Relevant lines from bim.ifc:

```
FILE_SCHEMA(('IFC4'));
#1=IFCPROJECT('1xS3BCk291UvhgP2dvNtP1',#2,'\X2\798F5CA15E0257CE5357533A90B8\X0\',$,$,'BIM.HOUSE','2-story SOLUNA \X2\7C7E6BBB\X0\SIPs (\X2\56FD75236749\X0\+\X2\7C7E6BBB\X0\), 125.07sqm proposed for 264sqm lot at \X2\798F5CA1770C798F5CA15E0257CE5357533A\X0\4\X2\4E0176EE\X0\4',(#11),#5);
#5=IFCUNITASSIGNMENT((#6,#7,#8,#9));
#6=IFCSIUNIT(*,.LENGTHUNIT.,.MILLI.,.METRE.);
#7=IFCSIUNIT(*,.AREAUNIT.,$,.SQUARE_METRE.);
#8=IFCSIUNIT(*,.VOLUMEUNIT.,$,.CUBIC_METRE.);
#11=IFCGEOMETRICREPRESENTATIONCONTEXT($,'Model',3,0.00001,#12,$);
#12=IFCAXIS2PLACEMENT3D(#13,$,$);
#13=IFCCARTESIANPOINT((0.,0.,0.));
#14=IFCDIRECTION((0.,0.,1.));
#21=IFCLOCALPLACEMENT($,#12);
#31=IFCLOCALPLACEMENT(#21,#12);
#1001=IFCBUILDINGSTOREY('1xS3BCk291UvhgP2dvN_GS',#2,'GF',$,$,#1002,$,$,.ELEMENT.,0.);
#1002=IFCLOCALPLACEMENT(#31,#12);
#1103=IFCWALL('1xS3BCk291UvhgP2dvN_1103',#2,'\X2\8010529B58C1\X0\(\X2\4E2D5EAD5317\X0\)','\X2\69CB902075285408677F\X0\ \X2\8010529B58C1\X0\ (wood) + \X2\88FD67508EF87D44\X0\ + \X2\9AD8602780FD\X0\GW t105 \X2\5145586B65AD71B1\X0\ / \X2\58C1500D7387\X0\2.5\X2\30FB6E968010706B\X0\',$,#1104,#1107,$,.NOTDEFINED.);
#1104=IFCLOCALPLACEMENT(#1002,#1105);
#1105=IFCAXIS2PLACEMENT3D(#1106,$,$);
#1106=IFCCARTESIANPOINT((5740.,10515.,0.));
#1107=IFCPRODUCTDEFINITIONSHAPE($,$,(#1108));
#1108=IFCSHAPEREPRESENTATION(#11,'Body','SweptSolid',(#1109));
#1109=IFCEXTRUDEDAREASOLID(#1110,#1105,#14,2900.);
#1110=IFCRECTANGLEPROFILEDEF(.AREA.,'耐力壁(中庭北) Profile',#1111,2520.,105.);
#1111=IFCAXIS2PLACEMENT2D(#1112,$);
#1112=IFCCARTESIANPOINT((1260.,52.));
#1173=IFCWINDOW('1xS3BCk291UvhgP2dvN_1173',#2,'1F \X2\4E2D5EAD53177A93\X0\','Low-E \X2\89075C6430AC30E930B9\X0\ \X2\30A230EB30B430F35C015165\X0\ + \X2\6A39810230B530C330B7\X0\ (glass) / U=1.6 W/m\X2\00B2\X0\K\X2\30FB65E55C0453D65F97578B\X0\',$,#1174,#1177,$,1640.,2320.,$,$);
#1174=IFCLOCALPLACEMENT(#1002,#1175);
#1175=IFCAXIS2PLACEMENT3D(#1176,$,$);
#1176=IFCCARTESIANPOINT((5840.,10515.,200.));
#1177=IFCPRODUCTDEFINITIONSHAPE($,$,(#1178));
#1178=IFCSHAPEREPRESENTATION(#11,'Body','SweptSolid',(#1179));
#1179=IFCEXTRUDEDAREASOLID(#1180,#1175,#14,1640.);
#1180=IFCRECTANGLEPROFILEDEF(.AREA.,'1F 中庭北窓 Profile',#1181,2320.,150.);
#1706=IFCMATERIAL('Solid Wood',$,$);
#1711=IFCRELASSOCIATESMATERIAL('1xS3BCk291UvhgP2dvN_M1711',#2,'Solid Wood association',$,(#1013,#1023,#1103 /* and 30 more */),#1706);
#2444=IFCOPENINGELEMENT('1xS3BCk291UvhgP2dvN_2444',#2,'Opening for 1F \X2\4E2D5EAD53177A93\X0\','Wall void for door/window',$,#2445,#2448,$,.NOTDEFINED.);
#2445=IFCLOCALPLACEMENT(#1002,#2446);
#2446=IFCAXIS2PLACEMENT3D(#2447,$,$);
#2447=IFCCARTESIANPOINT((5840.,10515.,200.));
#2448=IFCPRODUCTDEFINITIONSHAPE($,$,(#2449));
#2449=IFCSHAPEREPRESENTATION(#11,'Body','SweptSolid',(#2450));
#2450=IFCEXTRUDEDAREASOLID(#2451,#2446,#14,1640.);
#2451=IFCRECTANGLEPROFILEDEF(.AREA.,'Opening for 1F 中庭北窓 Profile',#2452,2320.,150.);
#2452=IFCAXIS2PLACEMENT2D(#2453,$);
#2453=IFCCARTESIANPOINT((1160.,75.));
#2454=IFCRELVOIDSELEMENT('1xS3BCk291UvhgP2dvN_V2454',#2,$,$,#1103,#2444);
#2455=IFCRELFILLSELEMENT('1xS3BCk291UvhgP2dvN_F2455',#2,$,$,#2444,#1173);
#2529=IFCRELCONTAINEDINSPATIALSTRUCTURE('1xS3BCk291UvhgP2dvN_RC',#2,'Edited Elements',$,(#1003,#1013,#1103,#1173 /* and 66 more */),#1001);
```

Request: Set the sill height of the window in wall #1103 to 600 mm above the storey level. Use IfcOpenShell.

```python
import numpy as np
import ifcopenshell
import ifcopenshell.api.geometry
import ifcopenshell.geom
import ifcopenshell.util.element
import ifcopenshell.util.placement
import ifcopenshell.util.shape
import ifcopenshell.util.unit

model = ifcopenshell.open("bim.ifc")
unit_scale = ifcopenshell.util.unit.calculate_unit_scale(model)

window = model.by_guid("1xS3BCk291UvhgP2dvN_1173")
opening = window.FillsVoids[0].RelatingOpeningElement
storey = ifcopenshell.util.element.get_container(window, ifc_class="IfcBuildingStorey")
level = ifcopenshell.util.placement.get_local_placement(storey.ObjectPlacement)[2, 3]

# The opening's origin need not be at the sill, so measure its lowest point.
shape = ifcopenshell.geom.create_shape(ifcopenshell.geom.settings(), opening)
bottom = ifcopenshell.util.shape.get_shape_bottom_elevation(shape, shape.geometry) / unit_scale
dz = level + 600.0 - bottom

shift = np.array([0.0, 0.0, dz])
# The window is not placed relative to its opening, so move both.
for product in (opening, window):
    matrix = ifcopenshell.util.placement.get_local_placement(product.ObjectPlacement)
    matrix[:3, 3] += shift
    ifcopenshell.api.geometry.edit_object_placement(model, product=product, matrix=matrix, is_si=False)

print(f"moved by {dz * unit_scale:+.3f} m")

model.write("bim-out.ifc")
```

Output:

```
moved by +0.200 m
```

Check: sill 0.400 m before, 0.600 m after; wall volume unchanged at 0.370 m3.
